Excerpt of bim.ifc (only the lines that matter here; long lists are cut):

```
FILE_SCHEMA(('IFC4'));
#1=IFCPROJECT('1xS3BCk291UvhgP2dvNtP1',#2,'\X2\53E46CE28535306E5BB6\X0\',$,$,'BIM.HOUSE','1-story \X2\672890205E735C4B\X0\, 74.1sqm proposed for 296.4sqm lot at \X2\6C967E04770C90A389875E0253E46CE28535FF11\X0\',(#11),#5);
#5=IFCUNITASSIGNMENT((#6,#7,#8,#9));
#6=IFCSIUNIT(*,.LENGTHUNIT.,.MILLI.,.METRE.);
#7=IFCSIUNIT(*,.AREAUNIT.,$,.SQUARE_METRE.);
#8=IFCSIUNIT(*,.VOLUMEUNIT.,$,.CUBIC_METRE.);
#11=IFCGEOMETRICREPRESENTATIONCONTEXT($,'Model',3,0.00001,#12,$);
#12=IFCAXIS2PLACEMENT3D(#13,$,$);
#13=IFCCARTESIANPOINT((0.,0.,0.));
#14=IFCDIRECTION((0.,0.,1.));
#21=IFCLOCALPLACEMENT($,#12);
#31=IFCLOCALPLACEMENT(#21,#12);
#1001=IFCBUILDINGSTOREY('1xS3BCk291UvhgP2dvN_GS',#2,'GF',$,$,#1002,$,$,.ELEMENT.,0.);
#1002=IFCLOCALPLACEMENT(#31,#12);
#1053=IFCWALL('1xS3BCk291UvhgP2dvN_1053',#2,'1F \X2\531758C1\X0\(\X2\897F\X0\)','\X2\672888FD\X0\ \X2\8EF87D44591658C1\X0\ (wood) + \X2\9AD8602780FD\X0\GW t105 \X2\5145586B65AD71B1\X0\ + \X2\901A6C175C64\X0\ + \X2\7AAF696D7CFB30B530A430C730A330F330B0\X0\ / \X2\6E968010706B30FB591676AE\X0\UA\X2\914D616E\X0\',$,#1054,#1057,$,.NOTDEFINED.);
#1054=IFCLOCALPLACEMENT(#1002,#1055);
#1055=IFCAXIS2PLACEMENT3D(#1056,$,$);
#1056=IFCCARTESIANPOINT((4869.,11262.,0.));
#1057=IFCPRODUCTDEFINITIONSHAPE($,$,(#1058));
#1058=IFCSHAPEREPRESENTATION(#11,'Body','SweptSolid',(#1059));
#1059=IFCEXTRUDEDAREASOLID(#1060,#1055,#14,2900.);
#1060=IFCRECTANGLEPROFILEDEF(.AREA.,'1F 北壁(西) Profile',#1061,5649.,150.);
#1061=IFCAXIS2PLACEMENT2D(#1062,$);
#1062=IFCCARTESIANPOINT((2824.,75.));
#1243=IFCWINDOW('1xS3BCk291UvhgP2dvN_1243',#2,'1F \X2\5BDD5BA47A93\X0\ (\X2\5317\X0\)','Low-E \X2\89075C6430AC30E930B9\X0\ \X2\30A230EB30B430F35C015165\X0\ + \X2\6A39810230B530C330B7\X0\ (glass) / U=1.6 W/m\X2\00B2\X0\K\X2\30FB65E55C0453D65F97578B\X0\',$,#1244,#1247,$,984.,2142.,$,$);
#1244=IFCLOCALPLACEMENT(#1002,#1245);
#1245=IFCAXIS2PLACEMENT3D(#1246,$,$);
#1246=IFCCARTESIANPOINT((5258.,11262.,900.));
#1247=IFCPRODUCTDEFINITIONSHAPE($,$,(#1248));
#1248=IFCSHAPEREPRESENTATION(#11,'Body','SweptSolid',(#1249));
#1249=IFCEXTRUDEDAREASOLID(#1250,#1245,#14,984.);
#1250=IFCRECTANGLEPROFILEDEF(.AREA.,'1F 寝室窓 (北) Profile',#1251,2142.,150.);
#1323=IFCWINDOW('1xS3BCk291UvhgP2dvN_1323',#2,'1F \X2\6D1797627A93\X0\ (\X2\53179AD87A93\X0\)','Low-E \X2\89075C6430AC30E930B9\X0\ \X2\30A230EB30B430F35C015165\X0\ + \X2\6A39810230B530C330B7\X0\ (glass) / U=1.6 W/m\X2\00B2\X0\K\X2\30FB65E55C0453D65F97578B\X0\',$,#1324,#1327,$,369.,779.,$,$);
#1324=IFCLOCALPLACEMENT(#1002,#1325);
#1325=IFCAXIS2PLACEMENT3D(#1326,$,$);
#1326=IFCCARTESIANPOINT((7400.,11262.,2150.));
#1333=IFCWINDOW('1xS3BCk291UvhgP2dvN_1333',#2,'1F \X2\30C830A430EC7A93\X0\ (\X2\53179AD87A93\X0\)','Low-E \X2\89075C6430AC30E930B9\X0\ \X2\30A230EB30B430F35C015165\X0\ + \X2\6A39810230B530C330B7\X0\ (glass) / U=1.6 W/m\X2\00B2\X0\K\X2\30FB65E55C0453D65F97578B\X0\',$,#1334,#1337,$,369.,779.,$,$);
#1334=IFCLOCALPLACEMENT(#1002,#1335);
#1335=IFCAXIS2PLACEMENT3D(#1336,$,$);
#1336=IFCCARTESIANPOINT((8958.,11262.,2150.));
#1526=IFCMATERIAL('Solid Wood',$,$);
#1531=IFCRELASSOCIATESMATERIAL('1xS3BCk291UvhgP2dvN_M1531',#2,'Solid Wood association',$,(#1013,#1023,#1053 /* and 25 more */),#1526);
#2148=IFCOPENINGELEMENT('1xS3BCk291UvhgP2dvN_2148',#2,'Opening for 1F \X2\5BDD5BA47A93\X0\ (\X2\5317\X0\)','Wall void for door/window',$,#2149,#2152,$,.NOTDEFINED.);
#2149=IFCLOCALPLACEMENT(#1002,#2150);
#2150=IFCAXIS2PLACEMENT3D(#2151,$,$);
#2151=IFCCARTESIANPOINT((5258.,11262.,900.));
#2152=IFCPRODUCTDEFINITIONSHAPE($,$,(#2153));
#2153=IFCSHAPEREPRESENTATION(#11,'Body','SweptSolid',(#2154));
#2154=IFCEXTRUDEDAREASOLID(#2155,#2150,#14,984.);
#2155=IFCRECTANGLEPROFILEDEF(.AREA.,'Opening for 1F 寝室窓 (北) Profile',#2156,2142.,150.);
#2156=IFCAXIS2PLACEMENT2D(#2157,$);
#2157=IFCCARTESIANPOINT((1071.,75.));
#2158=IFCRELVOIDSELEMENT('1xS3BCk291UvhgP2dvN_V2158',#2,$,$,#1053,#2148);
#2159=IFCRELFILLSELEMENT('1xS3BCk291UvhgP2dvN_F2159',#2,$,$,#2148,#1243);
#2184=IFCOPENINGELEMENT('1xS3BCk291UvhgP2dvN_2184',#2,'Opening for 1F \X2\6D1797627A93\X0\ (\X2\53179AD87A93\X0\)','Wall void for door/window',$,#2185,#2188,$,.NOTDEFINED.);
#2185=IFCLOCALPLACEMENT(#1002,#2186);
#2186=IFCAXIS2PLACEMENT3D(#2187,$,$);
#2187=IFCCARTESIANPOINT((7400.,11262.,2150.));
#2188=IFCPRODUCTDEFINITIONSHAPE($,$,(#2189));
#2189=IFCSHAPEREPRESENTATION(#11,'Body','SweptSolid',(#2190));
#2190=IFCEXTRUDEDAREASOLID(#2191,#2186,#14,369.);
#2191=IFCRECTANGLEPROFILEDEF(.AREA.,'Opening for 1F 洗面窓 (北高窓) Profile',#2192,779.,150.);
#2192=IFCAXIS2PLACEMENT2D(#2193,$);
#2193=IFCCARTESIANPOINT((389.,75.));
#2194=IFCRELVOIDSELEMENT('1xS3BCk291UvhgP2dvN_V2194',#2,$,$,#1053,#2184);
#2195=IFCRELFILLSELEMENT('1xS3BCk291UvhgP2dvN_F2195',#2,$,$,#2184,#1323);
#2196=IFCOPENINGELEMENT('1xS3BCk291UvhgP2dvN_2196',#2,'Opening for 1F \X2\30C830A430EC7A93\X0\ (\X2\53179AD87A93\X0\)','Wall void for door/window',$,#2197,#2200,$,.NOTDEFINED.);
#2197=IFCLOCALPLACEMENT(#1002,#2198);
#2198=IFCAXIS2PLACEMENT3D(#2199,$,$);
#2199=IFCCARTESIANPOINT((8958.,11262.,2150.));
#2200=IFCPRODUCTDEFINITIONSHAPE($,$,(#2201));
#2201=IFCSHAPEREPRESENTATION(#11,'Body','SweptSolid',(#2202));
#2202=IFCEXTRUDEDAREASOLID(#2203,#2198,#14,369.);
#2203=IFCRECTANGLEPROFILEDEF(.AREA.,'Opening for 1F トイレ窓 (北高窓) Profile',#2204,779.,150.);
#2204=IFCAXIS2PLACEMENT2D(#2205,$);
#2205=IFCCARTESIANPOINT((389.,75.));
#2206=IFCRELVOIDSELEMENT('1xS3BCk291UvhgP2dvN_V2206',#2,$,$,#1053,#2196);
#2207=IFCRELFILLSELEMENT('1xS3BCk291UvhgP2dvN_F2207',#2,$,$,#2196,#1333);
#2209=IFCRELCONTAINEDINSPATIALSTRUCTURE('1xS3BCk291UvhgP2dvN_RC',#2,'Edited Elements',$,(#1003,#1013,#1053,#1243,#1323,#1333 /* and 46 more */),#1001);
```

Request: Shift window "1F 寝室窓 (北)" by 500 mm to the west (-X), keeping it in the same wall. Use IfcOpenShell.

```python
import ifcopenshell
import ifcopenshell.api.geometry
import ifcopenshell.util.placement

model = ifcopenshell.open("bim.ifc")

window = model.by_guid("1xS3BCk291UvhgP2dvN_1243")
opening = window.FillsVoids[0].RelatingOpeningElement
wall = opening.VoidsElements[0].RelatingBuildingElement

wall_matrix = ifcopenshell.util.placement.get_local_placement(wall.ObjectPlacement)
shift = wall_matrix[:3, 0] * -500.0
before = ifcopenshell.util.placement.get_local_placement(window.ObjectPlacement)[:3, 3].copy()

# The window is not placed relative to its opening, so move both.
for product in (opening, window):
    matrix = ifcopenshell.util.placement.get_local_placement(product.ObjectPlacement)
    matrix[:3, 3] += shift
    ifcopenshell.api.geometry.edit_object_placement(model, product=product, matrix=matrix, is_si=False)

after = ifcopenshell.util.placement.get_local_placement(window.ObjectPlacement)[:3, 3]
print("window moved by", (after - before).round(3) + 0.0)

model.write("bim_v2.ifc")
```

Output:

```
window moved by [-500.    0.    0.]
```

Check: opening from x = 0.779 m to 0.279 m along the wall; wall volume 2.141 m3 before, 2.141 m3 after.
